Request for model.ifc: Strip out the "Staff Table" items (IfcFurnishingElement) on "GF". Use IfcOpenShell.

First a look at what the model holds.

```python
import ifcopenshell
import ifcopenshell.util.element

model = ifcopenshell.open("model.ifc")
print(model.schema)
storey = next(s for s in model.by_type("IfcBuildingStorey") if s.Name == "GF")
furniture = [e for e in ifcopenshell.util.element.get_decomposition(storey) if e.is_a("IfcFurnishingElement")]
seen = {}
for e in furniture:
    element_type = ifcopenshell.util.element.get_type(e)
    name = element_type.Name if element_type not in (None, e) else None
    seen[name] = seen.get(name, 0) + 1
for name, count in sorted(seen.items(), key=str):
    print(count, "x", name)
```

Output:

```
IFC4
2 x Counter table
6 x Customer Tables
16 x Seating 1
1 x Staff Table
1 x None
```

```python
import ifcopenshell
import ifcopenshell.api.root
import ifcopenshell.util.element

model = ifcopenshell.open("model.ifc")

storey = next(s for s in model.by_type("IfcBuildingStorey") if s.Name == "GF")
furniture = [e for e in ifcopenshell.util.element.get_decomposition(storey) if e.is_a("IfcFurnishingElement")]
targets = [e for e in furniture if (t := ifcopenshell.util.element.get_type(e)) not in (None, e) and t.Name == "Staff Table"]

for e in targets:
    ifcopenshell.api.root.remove_product(model, product=e)
print(len(targets), "removed")

model.write("model_v2.ifc")
```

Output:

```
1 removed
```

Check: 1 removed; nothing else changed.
